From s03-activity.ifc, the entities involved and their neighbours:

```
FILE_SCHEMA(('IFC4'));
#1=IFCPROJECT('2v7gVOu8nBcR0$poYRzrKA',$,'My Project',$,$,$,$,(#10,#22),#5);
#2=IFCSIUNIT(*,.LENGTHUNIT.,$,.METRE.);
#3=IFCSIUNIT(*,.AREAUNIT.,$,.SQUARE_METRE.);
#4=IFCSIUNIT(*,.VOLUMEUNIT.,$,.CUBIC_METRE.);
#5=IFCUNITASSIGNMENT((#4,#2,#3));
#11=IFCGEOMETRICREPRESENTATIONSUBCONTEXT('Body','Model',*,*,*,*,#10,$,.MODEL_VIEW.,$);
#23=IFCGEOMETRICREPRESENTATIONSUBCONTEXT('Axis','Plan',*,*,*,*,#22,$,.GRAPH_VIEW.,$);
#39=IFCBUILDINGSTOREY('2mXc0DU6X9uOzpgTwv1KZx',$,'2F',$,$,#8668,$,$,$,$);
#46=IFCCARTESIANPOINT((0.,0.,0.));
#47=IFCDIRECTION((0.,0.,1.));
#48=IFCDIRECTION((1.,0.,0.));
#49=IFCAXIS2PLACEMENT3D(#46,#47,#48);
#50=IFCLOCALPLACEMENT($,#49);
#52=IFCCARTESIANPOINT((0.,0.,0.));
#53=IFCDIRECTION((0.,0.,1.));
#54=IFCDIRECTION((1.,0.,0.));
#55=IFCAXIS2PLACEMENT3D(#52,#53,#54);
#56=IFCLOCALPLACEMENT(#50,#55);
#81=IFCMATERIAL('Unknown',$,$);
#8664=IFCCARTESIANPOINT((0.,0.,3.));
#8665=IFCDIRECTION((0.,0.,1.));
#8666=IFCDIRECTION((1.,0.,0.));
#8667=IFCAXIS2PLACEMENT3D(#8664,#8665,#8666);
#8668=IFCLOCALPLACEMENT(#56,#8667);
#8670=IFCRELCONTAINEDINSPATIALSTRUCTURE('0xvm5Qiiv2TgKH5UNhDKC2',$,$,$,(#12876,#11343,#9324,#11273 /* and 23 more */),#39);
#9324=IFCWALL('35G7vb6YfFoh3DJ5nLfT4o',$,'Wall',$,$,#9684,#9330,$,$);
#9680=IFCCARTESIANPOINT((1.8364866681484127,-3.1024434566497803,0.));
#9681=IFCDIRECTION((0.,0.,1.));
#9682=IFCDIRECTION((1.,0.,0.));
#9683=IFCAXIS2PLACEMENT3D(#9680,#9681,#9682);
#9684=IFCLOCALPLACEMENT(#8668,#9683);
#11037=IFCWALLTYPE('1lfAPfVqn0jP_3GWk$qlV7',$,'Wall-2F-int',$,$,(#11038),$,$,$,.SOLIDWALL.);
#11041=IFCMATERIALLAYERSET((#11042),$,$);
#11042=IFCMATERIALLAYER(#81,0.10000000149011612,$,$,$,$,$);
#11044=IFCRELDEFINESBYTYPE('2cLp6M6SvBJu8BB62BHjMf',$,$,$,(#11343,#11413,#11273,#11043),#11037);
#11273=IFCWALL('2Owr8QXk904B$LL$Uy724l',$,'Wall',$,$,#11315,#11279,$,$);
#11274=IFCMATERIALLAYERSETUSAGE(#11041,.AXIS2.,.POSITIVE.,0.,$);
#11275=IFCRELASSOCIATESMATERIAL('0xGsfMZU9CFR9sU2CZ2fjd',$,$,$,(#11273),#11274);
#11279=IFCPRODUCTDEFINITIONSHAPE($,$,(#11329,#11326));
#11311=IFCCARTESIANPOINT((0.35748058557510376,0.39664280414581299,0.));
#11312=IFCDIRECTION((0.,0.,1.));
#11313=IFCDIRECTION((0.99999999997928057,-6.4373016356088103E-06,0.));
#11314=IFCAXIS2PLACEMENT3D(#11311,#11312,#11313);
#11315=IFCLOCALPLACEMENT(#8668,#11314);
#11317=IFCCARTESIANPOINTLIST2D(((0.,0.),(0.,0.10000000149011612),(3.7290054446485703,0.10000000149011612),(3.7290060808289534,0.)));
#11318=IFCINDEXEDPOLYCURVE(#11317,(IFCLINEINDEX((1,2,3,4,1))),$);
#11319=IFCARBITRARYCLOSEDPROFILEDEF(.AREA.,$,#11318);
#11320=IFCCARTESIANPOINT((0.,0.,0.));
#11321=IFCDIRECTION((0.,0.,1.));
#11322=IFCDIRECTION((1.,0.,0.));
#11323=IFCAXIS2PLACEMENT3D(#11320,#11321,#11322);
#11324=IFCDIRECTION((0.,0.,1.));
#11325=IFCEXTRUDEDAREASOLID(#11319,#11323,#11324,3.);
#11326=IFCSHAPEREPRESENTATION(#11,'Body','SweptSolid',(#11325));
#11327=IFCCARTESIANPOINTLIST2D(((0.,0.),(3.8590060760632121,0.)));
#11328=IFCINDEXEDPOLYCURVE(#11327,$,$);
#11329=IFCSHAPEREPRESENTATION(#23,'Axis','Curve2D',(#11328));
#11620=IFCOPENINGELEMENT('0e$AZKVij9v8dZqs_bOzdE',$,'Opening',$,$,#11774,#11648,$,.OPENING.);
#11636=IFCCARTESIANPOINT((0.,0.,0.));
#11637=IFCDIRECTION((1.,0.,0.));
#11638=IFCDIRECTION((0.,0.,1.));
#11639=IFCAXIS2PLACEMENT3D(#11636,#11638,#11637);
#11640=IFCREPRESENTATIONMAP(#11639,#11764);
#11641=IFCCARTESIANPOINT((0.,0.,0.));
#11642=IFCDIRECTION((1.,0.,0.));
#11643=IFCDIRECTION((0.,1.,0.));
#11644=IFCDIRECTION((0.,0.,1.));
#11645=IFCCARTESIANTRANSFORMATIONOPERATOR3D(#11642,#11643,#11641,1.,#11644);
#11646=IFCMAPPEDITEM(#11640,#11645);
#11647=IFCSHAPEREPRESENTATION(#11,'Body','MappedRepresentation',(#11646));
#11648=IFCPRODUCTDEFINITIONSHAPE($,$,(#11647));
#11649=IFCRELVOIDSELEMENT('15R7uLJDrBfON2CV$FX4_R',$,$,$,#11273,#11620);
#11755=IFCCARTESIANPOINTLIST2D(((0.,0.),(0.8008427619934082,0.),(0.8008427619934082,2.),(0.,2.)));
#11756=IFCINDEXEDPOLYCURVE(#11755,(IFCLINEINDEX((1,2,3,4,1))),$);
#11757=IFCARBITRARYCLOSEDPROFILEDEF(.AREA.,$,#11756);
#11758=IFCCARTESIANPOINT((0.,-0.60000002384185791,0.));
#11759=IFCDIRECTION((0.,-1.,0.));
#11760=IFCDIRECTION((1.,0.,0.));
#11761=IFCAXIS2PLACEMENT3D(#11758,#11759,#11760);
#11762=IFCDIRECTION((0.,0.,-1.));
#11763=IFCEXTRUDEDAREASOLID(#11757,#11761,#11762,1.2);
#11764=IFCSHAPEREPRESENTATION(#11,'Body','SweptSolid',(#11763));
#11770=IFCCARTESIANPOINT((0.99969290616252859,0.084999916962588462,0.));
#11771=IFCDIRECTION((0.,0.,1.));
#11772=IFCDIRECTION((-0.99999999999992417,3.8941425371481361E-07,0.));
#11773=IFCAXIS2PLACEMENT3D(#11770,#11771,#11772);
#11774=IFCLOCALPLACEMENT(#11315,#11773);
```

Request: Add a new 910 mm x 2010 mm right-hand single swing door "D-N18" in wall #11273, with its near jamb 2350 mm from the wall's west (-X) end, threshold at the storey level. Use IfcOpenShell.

```python
import numpy as np
import ifcopenshell
import ifcopenshell.api.feature
import ifcopenshell.api.geometry
import ifcopenshell.api.root
import ifcopenshell.api.spatial
import ifcopenshell.geom
import ifcopenshell.util.element
import ifcopenshell.util.placement
import ifcopenshell.util.representation
import ifcopenshell.util.shape
import ifcopenshell.util.unit

model = ifcopenshell.open("s03-activity.ifc")
unit_scale = ifcopenshell.util.unit.calculate_unit_scale(model)
settings = ifcopenshell.geom.settings()


def volume(element):
    """Net volume in cubic metres, openings subtracted."""
    shape = ifcopenshell.geom.create_shape(settings, element)
    return ifcopenshell.util.shape.get_volume(shape.geometry)


wall = model.by_guid("2Owr8QXk904B$LL$Uy724l")
storey = ifcopenshell.util.element.get_container(wall, ifc_class="IfcBuildingStorey")
context = ifcopenshell.util.representation.get_context(model, "Model", "Body", "MODEL_VIEW")
before = volume(wall)

width, height, from_end, sill = 0.91, 2.01, 2.35, 0.0  # metres

# The wall runs along its own X axis, and the end named is its -X end.
wall_shape = ifcopenshell.geom.create_shape(settings, wall)
x, y, z = ifcopenshell.util.shape.get_vertices(wall_shape.geometry).T
start = x.min() + from_end
face, thickness = float(y.min()), float(y.max() - y.min())
wall_matrix = ifcopenshell.util.placement.get_local_placement(wall.ObjectPlacement)
level = ifcopenshell.util.placement.get_local_placement(storey.ObjectPlacement)[2, 3]


def in_wall(x, y):
    """Placement at x, y metres in the wall's axes, at sill height."""
    matrix = wall_matrix.copy()
    matrix[:, 3] = wall_matrix @ np.array([x / unit_scale, y / unit_scale, 0.0, 1.0])
    matrix[2, 3] = level + sill / unit_scale
    return matrix


# Opening: a box that overshoots both wall faces by 50 mm.
opening = ifcopenshell.api.root.create_entity(model, ifc_class="IfcOpeningElement", predefined_type="OPENING")
box = ifcopenshell.api.geometry.add_wall_representation(
    model, context=context, length=width, height=height, thickness=thickness + 0.1
)
ifcopenshell.api.geometry.assign_representation(model, product=opening, representation=box)
ifcopenshell.api.geometry.edit_object_placement(model, product=opening, matrix=in_wall(start, face - 0.05), is_si=False)
ifcopenshell.api.feature.add_feature(model, feature=opening, element=wall)

door = ifcopenshell.api.root.create_entity(model, ifc_class="IfcDoor", name="D-N18", predefined_type="DOOR")
door.OverallWidth, door.OverallHeight = width / unit_scale, height / unit_scale
door.OperationType = "SINGLE_SWING_RIGHT"
body = ifcopenshell.api.geometry.add_door_representation(
    model,
    context=context,
    overall_width=door.OverallWidth,
    overall_height=door.OverallHeight,
    operation_type="SINGLE_SWING_RIGHT",
    lining_properties={"LiningDepth": thickness / unit_scale, "ThresholdDepth": thickness / unit_scale},
)
ifcopenshell.api.geometry.assign_representation(model, product=door, representation=body)
ifcopenshell.api.spatial.assign_container(model, products=[door], relating_structure=storey)
ifcopenshell.api.feature.add_filling(model, opening=opening, element=door)

# The lining spans the wall, so the door starts at the wall face.
ifcopenshell.api.geometry.edit_object_placement(model, product=door, matrix=in_wall(start, face), is_si=False)

after = volume(wall)

print(f"wall volume {before:.3f} -> {after:.3f} m3")

model.write("s03-activity-out.ifc")
```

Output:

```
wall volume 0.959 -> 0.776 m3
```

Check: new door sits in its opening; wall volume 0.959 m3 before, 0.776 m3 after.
